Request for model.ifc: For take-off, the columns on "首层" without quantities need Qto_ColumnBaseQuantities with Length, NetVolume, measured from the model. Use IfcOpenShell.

First a look at what the model holds.

```python
import ifcopenshell
import ifcopenshell.util.element
import ifcopenshell.util.unit

model = ifcopenshell.open("model.ifc")
print(model.schema)
for unit_type in ("LENGTHUNIT", "AREAUNIT", "VOLUMEUNIT"):
    print(unit_type, ifcopenshell.util.unit.calculate_unit_scale(model, unit_type))
storey = next(s for s in model.by_type("IfcBuildingStorey") if s.Name == "首层")
columns = [e for e in ifcopenshell.util.element.get_decomposition(storey) if e.is_a("IfcColumn")]
for e in sorted(columns, key=lambda e: e.id()):
    print(e.id(), e.is_a(), e.Name, list(ifcopenshell.util.element.get_psets(e, qtos_only=True)), sep=" | ")
```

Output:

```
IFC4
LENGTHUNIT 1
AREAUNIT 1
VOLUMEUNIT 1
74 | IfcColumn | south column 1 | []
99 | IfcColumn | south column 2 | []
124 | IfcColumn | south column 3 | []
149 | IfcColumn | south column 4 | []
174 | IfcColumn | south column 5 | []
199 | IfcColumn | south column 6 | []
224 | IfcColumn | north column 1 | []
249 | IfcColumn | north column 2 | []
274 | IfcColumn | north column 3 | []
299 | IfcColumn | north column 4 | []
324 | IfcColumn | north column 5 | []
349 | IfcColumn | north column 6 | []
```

```python
import ifcopenshell
import ifcopenshell.api.pset
import ifcopenshell.geom
import ifcopenshell.util.element
import ifcopenshell.util.shape
import ifcopenshell.util.unit

model = ifcopenshell.open("model.ifc")
unit_scale = ifcopenshell.util.unit.calculate_unit_scale(model)
volume_scale = ifcopenshell.util.unit.calculate_unit_scale(model, "VOLUMEUNIT")
settings = ifcopenshell.geom.settings()

storey = next(s for s in model.by_type("IfcBuildingStorey") if s.Name == "首层")
columns = [e for e in ifcopenshell.util.element.get_decomposition(storey) if e.is_a("IfcColumn")]

for e in sorted(columns, key=lambda e: e.id()):
    if ifcopenshell.util.element.get_psets(e, qtos_only=True, should_inherit=False):
        continue
    # Geometry comes back in metres, in the element's own axes.
    shape = ifcopenshell.geom.create_shape(settings, e)
    values = {
        "Length": ifcopenshell.util.shape.get_z(shape.geometry) / unit_scale,
        "NetVolume": ifcopenshell.util.shape.get_volume(shape.geometry) / volume_scale,
    }
    qto = ifcopenshell.api.pset.add_qto(model, product=e, name="Qto_ColumnBaseQuantities")
    ifcopenshell.api.pset.edit_qto(model, qto=qto, properties=values)
    print(e.id(), {k: round(v, 3) for k, v in values.items()})

model.write("model_v2.ifc")
```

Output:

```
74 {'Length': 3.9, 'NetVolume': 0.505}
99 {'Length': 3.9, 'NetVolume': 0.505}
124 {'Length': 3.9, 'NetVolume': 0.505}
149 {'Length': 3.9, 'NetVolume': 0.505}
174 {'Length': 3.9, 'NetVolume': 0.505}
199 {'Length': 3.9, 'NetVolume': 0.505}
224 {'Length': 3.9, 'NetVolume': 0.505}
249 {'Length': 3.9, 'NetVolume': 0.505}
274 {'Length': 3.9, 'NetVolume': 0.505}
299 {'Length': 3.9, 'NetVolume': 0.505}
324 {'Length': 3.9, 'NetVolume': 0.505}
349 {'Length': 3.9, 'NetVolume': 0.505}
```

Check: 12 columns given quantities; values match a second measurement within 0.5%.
